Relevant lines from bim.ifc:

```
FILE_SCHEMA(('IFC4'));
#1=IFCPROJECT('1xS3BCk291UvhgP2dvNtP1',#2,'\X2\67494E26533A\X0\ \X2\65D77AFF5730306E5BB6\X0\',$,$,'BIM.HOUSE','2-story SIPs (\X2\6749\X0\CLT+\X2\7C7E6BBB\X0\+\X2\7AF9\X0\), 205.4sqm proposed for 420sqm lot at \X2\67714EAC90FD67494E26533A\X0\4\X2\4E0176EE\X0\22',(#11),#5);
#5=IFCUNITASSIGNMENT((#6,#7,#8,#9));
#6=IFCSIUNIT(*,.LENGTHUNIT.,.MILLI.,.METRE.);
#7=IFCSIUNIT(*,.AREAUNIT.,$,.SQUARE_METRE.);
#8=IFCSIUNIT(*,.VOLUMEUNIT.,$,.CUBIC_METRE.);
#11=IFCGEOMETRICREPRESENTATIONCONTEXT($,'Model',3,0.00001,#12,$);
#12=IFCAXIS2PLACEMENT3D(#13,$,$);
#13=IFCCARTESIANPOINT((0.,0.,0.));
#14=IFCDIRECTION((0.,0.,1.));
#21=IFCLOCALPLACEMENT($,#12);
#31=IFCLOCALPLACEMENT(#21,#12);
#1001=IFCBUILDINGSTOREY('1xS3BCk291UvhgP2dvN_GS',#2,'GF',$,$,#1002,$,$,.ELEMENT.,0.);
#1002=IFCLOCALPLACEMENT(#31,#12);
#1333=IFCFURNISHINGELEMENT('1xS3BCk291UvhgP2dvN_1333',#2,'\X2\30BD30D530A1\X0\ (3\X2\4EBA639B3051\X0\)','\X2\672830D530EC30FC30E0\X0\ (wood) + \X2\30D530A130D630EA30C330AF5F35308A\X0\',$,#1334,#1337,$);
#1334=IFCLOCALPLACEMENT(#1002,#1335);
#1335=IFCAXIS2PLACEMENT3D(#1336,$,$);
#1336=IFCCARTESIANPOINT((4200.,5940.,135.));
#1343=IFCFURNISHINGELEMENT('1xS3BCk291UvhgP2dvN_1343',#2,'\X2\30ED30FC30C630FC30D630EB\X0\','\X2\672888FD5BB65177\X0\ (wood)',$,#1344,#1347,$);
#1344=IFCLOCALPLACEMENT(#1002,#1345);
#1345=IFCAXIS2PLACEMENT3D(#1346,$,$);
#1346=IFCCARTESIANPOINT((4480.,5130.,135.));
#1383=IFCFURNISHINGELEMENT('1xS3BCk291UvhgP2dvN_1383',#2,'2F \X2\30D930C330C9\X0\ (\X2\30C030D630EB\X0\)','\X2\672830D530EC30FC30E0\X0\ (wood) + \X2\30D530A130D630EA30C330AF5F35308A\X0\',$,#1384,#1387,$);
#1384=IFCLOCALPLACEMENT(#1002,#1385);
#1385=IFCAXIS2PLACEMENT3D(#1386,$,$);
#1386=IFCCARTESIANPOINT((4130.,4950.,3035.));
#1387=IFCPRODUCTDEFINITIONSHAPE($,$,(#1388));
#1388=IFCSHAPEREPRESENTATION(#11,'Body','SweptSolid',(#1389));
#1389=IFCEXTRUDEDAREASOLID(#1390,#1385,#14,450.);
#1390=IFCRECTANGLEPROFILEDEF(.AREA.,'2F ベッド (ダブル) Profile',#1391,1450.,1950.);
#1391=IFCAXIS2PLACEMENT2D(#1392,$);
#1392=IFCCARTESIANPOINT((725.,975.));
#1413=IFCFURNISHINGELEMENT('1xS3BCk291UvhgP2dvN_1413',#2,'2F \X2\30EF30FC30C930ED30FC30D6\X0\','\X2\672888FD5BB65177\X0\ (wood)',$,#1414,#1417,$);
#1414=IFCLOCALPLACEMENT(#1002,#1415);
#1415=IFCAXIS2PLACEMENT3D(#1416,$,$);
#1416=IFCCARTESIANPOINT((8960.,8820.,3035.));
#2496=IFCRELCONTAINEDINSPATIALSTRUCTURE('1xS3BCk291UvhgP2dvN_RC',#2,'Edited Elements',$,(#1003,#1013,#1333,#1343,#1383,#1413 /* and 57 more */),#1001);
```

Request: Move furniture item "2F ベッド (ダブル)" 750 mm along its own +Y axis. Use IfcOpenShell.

```python
import ifcopenshell
import ifcopenshell.api.geometry
import ifcopenshell.util.placement

model = ifcopenshell.open("bim.ifc")

item = model.by_guid("1xS3BCk291UvhgP2dvN_1383")
matrix = ifcopenshell.util.placement.get_local_placement(item.ObjectPlacement)
matrix[:3, 3] += matrix[:3, 1] * 750.0
ifcopenshell.api.geometry.edit_object_placement(model, product=item, matrix=matrix, is_si=False)

print(ifcopenshell.util.placement.get_local_placement(item.ObjectPlacement).round(3) + 0.0)

model.write("bim_edited.ifc")
```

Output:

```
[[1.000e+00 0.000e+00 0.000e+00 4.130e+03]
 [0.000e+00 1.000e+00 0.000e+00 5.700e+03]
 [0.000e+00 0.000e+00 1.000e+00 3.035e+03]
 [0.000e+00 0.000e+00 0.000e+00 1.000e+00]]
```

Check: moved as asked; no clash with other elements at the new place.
